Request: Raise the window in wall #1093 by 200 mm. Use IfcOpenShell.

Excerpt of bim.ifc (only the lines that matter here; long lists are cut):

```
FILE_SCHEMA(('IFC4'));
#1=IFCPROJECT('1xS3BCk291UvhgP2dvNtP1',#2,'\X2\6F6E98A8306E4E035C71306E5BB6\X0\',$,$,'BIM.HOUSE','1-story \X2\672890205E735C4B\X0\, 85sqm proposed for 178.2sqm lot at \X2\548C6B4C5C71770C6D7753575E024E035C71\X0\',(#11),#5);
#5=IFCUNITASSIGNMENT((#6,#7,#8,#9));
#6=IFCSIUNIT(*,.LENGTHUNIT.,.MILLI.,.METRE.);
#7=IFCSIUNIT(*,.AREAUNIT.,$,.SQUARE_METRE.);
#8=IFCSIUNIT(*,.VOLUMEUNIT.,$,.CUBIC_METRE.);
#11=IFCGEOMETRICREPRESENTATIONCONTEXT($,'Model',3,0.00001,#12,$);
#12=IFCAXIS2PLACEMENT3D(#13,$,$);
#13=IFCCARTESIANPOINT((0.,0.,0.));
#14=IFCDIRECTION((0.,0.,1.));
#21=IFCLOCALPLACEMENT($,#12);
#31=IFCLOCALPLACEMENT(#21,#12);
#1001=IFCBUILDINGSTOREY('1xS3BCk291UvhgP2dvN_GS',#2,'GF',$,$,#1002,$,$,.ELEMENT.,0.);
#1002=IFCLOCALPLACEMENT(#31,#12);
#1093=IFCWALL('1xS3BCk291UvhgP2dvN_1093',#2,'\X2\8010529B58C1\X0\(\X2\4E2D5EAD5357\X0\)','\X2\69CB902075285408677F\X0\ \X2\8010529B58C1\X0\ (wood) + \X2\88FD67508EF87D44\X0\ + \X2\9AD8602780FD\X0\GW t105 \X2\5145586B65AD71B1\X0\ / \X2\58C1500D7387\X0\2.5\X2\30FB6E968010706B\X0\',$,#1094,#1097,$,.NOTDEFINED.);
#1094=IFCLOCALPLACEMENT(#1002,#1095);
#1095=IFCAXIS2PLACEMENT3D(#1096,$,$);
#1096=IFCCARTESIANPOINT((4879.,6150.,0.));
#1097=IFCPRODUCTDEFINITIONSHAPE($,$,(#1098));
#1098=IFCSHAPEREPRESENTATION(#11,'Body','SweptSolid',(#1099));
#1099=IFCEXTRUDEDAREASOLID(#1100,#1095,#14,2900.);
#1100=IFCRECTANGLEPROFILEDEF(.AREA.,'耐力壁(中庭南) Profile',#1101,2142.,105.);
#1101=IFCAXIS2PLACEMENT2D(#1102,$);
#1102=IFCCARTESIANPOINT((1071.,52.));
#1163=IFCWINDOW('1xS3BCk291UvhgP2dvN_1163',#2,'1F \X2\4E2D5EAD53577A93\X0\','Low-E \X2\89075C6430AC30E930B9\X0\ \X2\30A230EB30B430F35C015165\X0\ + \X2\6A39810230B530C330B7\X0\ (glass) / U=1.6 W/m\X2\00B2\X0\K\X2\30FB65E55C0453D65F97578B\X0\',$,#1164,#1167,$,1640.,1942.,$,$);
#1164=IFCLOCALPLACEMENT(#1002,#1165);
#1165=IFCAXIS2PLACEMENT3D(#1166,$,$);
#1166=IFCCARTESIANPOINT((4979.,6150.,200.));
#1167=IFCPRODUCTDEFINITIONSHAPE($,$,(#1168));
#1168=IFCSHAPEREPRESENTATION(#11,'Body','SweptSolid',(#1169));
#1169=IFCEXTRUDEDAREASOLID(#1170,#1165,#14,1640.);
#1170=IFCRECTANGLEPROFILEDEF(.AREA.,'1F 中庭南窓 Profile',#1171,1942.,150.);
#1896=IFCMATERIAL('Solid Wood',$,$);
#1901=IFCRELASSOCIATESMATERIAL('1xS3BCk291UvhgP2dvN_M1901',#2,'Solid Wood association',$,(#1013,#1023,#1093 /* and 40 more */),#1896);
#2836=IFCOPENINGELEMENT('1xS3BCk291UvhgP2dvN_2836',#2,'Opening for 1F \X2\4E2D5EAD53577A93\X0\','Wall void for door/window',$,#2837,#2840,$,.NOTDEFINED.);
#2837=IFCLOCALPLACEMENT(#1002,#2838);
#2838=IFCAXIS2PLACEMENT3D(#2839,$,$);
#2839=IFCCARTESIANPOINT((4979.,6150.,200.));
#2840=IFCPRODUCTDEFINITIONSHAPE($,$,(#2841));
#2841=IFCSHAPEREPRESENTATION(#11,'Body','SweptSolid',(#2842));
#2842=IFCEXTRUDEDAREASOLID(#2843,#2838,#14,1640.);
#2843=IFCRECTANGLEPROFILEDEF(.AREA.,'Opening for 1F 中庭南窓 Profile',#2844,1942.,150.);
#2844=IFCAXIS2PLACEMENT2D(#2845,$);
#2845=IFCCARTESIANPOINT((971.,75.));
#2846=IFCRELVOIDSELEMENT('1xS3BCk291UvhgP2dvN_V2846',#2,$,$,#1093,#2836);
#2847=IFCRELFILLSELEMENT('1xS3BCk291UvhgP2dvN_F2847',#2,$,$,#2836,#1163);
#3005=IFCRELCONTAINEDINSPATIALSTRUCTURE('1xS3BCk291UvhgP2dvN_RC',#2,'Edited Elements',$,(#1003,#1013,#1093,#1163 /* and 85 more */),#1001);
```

```python
import numpy as np
import ifcopenshell
import ifcopenshell.api.geometry
import ifcopenshell.util.placement
import ifcopenshell.util.unit

model = ifcopenshell.open("bim.ifc")
unit_scale = ifcopenshell.util.unit.calculate_unit_scale(model)

window = model.by_guid("1xS3BCk291UvhgP2dvN_1163")
opening = window.FillsVoids[0].RelatingOpeningElement
dz = 200.0

shift = np.array([0.0, 0.0, dz])
# The window is not placed relative to its opening, so move both.
for product in (opening, window):
    matrix = ifcopenshell.util.placement.get_local_placement(product.ObjectPlacement)
    matrix[:3, 3] += shift
    ifcopenshell.api.geometry.edit_object_placement(model, product=product, matrix=matrix, is_si=False)

print(f"moved by {dz * unit_scale:+.3f} m")

model.write("bim_v2.ifc")
```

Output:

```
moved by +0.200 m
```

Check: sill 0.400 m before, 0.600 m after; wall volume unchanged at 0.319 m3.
